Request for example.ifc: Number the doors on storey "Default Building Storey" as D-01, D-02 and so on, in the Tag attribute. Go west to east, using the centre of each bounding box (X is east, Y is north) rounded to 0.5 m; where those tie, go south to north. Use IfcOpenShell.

First a look at what the model holds.

```python
import ifcopenshell
import ifcopenshell.util.element
import ifcopenshell.util.placement

model = ifcopenshell.open("example.ifc")
print(model.schema)
storey = next(s for s in model.by_type("IfcBuildingStorey") if s.Name == "Default Building Storey")
doors = [e for e in ifcopenshell.util.element.get_decomposition(storey) if e.is_a("IfcDoor")]
for e in sorted(doors, key=lambda e: e.id()):
    origin = ifcopenshell.util.placement.get_local_placement(e.ObjectPlacement)[:3, 3]
    print(e.id(), e.Tag, e.Name, origin.round(2) + 0.0, sep=" | ")
```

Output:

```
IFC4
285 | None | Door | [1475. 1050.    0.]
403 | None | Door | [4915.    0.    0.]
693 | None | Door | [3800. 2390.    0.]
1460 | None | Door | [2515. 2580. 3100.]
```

```python
import ifcopenshell
import ifcopenshell.geom
import ifcopenshell.util.element
import ifcopenshell.util.shape

model = ifcopenshell.open("example.ifc")
settings = ifcopenshell.geom.settings()
settings.set("use-world-coords", True)


def centre(element):
    shape = ifcopenshell.geom.create_shape(settings, element)
    return ifcopenshell.util.shape.get_bbox_centroid(shape.geometry)


storey = next(s for s in model.by_type("IfcBuildingStorey") if s.Name == "Default Building Storey")
doors = [e for e in ifcopenshell.util.element.get_decomposition(storey) if e.is_a("IfcDoor")]

# Insertion points can sit at a corner or the storey origin, so sort by the geometry (in metres).
centres = {e: centre(e) for e in doors}
doors.sort(key=lambda e: (round(centres[e][0] / 0.5), centres[e][1]))

for i, e in enumerate(doors, start=1):
    number = f"D-{i:02d}"
    e.Tag = number
    print(e.id(), number)

model.write("example_edited.ifc")
```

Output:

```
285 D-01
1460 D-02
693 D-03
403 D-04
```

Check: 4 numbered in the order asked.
